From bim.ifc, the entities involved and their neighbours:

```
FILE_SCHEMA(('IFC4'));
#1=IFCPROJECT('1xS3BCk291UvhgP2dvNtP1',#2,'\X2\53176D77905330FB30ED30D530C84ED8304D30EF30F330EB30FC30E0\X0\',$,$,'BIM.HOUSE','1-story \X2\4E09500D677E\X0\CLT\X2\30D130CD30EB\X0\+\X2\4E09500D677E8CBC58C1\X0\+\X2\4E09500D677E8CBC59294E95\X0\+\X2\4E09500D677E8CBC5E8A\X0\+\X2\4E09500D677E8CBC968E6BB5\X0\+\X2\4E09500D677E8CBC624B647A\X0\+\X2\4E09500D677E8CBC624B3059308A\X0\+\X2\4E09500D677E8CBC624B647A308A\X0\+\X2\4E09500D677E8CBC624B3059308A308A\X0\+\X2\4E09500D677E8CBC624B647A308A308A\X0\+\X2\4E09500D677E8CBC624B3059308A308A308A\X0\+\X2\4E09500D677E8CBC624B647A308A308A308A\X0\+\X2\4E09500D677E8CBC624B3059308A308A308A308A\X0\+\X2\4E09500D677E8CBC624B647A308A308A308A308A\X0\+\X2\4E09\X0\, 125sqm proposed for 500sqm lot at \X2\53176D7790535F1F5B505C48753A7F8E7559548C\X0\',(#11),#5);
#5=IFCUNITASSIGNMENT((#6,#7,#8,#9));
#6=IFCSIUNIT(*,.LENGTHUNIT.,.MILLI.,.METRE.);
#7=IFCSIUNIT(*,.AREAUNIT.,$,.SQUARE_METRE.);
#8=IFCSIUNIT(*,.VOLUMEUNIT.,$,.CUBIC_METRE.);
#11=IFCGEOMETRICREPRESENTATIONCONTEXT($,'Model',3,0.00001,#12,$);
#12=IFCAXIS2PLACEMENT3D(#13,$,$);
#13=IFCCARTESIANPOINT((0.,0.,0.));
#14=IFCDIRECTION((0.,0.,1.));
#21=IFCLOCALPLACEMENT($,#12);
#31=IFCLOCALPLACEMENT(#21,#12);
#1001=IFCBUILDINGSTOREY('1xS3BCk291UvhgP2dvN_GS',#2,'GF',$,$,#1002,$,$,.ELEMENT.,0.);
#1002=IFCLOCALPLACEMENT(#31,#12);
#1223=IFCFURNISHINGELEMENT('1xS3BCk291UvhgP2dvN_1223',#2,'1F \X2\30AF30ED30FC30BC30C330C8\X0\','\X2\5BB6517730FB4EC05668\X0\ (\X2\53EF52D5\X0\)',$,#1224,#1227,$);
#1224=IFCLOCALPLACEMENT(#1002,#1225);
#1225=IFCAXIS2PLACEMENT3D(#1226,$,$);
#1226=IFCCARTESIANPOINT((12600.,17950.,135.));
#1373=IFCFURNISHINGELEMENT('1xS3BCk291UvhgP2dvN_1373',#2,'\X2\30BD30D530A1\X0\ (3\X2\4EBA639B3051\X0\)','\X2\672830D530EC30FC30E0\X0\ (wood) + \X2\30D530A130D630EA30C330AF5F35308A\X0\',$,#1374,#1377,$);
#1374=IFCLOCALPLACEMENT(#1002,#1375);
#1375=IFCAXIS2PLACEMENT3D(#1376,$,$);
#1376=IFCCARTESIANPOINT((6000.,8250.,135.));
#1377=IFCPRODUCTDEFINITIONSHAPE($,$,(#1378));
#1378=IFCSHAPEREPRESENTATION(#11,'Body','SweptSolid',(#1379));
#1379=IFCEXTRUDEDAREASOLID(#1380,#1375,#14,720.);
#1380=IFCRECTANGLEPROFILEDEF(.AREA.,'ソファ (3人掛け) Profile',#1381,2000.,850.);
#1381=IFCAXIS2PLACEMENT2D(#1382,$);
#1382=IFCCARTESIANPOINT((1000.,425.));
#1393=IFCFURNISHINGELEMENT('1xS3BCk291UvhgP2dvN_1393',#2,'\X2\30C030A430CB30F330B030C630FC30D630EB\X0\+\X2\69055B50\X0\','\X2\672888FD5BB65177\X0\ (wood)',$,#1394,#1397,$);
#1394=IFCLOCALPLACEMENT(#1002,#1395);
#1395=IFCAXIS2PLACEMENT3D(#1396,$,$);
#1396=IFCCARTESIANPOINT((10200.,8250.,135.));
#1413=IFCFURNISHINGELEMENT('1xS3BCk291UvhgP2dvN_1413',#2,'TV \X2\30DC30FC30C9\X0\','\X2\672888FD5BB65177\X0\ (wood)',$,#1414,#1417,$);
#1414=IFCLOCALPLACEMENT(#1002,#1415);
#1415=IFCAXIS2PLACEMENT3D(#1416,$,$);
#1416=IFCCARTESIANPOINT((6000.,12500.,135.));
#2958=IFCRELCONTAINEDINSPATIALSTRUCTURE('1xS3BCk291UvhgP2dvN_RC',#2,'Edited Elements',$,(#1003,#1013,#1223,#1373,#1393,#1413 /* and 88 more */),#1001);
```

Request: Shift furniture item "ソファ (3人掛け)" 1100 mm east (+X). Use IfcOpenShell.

```python
import ifcopenshell
import ifcopenshell.api.geometry
import ifcopenshell.util.placement

model = ifcopenshell.open("bim.ifc")

item = model.by_guid("1xS3BCk291UvhgP2dvN_1373")
matrix = ifcopenshell.util.placement.get_local_placement(item.ObjectPlacement)
matrix[0, 3] += 1100.0
ifcopenshell.api.geometry.edit_object_placement(model, product=item, matrix=matrix, is_si=False)

print(ifcopenshell.util.placement.get_local_placement(item.ObjectPlacement).round(3) + 0.0)

model.write("bim_updated.ifc")
```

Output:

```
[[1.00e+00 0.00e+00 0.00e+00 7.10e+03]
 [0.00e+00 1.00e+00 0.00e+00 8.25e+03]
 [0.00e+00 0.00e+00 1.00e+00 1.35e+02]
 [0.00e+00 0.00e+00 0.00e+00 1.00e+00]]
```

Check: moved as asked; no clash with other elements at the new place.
